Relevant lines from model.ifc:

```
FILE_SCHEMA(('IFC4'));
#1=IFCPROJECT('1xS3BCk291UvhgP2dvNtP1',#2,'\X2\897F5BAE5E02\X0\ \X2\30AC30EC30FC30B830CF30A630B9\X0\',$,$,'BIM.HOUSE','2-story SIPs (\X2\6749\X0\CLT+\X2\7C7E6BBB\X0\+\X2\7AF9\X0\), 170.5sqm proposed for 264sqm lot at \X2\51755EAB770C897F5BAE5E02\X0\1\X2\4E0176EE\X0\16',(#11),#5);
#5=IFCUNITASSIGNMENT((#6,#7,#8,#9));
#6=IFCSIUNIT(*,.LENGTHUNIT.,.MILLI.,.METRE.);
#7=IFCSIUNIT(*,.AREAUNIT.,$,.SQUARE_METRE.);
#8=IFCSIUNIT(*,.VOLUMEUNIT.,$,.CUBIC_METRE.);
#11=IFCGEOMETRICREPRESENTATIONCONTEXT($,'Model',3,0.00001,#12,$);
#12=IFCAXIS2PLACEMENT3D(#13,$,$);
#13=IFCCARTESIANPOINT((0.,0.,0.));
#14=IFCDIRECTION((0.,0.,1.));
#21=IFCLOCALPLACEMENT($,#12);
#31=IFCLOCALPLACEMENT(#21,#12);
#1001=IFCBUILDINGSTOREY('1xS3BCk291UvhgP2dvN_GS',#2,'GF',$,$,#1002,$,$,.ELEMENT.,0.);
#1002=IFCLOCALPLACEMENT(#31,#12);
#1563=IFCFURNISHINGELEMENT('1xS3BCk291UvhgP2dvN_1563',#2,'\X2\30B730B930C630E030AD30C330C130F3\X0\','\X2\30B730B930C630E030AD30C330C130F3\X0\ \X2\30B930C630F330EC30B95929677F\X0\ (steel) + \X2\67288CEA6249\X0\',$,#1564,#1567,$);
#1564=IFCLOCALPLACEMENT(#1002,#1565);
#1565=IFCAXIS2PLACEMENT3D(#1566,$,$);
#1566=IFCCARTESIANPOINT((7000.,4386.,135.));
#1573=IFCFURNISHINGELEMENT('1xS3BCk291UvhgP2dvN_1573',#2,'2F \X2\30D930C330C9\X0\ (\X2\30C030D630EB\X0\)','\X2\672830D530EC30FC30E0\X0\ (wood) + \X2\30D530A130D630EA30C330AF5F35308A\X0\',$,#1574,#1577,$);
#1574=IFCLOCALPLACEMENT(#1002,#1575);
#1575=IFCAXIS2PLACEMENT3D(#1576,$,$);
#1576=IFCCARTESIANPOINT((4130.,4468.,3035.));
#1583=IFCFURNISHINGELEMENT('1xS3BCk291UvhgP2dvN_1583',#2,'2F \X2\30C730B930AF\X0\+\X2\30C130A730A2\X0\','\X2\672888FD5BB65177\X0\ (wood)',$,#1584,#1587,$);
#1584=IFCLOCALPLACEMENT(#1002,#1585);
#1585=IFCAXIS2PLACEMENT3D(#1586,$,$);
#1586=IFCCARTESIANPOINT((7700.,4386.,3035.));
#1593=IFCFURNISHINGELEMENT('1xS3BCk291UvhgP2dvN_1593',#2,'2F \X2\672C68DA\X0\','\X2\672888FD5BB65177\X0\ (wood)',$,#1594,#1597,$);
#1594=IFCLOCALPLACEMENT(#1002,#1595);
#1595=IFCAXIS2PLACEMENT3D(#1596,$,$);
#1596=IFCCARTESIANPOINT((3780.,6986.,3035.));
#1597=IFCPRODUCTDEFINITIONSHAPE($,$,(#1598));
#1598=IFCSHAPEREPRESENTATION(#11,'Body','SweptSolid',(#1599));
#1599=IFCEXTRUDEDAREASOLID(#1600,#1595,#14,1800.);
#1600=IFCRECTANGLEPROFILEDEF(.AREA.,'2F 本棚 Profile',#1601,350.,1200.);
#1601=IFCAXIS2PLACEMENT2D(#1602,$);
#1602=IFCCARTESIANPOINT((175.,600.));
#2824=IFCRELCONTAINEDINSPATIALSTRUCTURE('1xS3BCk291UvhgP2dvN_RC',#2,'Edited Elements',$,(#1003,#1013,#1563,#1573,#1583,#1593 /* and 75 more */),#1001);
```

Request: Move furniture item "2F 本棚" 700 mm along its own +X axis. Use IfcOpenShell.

```python
import ifcopenshell
import ifcopenshell.api.geometry
import ifcopenshell.util.placement
import ifcopenshell.util.unit

model = ifcopenshell.open("model.ifc")
unit_scale = ifcopenshell.util.unit.calculate_unit_scale(model)

item = model.by_id(1593)
matrix = ifcopenshell.util.placement.get_local_placement(item.ObjectPlacement)
matrix[:3, 3] += matrix[:3, 0] * 0.7 / unit_scale
ifcopenshell.api.geometry.edit_object_placement(model, product=item, matrix=matrix, is_si=False)

print(ifcopenshell.util.placement.get_local_placement(item.ObjectPlacement).round(3) + 0.0)

model.write("model_v2.ifc")
```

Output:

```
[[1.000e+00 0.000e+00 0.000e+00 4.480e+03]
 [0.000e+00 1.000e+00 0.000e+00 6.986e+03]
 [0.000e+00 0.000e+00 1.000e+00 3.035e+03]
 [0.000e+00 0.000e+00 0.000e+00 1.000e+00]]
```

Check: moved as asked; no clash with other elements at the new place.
